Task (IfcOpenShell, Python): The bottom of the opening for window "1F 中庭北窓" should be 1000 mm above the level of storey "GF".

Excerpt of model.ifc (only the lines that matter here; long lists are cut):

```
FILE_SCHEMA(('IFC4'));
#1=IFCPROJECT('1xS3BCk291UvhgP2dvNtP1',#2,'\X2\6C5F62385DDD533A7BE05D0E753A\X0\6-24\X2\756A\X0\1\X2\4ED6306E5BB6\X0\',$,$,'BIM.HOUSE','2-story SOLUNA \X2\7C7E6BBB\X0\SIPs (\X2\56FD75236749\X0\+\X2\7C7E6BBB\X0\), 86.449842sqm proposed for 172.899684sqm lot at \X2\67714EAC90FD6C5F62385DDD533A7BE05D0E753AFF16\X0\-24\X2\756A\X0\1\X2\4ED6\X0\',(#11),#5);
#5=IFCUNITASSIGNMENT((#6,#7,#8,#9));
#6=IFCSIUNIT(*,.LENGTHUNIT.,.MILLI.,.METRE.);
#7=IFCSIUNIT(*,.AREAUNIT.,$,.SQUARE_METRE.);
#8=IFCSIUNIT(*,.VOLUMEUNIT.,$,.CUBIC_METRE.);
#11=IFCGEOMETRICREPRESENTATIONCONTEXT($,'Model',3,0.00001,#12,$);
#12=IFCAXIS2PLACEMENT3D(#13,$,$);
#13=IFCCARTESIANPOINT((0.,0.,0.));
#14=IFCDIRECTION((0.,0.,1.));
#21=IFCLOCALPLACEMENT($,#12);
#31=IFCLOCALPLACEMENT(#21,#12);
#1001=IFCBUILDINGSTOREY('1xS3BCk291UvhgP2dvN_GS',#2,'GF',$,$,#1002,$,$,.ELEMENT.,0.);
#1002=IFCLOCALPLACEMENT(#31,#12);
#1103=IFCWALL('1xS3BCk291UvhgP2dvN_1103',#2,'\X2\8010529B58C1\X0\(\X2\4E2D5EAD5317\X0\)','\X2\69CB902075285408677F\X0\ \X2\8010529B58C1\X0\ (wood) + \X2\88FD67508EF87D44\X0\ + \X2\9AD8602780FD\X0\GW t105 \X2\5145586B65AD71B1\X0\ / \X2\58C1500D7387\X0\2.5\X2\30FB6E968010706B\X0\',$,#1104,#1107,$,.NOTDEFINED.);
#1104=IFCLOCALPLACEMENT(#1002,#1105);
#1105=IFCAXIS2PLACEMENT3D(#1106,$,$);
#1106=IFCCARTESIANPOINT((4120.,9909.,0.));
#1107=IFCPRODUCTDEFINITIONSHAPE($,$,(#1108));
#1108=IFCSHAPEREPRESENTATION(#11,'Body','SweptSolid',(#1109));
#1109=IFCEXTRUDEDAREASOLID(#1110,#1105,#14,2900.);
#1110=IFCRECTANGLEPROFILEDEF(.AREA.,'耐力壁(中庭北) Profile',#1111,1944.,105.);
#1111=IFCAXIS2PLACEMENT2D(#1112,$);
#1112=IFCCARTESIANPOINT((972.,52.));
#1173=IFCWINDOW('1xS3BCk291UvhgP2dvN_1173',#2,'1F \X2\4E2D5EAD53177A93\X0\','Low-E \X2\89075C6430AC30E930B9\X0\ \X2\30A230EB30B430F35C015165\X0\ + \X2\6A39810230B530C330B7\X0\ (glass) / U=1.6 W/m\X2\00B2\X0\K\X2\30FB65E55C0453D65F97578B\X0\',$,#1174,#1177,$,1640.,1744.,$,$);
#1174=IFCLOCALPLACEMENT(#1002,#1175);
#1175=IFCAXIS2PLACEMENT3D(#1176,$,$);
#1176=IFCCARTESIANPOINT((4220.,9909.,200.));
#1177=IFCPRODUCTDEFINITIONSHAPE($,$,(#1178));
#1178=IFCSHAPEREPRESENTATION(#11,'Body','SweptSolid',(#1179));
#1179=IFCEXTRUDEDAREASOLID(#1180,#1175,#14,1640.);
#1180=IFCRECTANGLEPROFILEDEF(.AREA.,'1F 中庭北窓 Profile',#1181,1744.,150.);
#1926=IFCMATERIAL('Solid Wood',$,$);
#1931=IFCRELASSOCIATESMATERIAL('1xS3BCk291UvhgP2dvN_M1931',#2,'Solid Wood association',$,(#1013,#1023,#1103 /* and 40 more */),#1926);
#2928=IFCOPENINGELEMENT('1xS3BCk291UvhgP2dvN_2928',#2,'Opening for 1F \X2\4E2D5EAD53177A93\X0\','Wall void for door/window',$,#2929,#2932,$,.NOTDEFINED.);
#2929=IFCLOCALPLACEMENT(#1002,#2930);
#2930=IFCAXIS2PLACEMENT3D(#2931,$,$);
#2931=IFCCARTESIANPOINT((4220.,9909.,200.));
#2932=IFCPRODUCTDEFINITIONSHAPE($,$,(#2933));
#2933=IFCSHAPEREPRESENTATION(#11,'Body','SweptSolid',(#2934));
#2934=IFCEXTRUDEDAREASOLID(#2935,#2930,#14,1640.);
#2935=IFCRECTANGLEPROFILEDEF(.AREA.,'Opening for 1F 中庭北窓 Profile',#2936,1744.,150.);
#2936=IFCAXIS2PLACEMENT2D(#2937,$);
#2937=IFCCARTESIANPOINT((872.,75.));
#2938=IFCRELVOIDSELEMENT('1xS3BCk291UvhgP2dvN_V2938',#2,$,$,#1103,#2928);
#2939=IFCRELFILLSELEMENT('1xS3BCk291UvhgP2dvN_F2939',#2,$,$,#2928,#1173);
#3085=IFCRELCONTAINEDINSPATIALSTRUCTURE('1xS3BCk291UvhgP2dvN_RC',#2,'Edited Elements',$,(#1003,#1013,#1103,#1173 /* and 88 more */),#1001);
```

```python
import numpy as np
import ifcopenshell
import ifcopenshell.api.geometry
import ifcopenshell.geom
import ifcopenshell.util.element
import ifcopenshell.util.placement
import ifcopenshell.util.shape
import ifcopenshell.util.unit

model = ifcopenshell.open("model.ifc")
unit_scale = ifcopenshell.util.unit.calculate_unit_scale(model)

window = model.by_guid("1xS3BCk291UvhgP2dvN_1173")
opening = window.FillsVoids[0].RelatingOpeningElement
storey = ifcopenshell.util.element.get_container(window, ifc_class="IfcBuildingStorey")
level = ifcopenshell.util.placement.get_local_placement(storey.ObjectPlacement)[2, 3]

# The opening's origin need not be at the sill, so measure its lowest point.
shape = ifcopenshell.geom.create_shape(ifcopenshell.geom.settings(), opening)
bottom = ifcopenshell.util.shape.get_shape_bottom_elevation(shape, shape.geometry) / unit_scale
dz = level + 1 / unit_scale - bottom

shift = np.array([0.0, 0.0, dz])
# The window is not placed relative to its opening, so move both.
for product in (opening, window):
    matrix = ifcopenshell.util.placement.get_local_placement(product.ObjectPlacement)
    matrix[:3, 3] += shift
    ifcopenshell.api.geometry.edit_object_placement(model, product=product, matrix=matrix, is_si=False)

print(f"moved by {dz * unit_scale:+.3f} m")

model.write("model_edited.ifc")
```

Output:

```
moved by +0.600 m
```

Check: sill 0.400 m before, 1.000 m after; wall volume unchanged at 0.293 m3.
